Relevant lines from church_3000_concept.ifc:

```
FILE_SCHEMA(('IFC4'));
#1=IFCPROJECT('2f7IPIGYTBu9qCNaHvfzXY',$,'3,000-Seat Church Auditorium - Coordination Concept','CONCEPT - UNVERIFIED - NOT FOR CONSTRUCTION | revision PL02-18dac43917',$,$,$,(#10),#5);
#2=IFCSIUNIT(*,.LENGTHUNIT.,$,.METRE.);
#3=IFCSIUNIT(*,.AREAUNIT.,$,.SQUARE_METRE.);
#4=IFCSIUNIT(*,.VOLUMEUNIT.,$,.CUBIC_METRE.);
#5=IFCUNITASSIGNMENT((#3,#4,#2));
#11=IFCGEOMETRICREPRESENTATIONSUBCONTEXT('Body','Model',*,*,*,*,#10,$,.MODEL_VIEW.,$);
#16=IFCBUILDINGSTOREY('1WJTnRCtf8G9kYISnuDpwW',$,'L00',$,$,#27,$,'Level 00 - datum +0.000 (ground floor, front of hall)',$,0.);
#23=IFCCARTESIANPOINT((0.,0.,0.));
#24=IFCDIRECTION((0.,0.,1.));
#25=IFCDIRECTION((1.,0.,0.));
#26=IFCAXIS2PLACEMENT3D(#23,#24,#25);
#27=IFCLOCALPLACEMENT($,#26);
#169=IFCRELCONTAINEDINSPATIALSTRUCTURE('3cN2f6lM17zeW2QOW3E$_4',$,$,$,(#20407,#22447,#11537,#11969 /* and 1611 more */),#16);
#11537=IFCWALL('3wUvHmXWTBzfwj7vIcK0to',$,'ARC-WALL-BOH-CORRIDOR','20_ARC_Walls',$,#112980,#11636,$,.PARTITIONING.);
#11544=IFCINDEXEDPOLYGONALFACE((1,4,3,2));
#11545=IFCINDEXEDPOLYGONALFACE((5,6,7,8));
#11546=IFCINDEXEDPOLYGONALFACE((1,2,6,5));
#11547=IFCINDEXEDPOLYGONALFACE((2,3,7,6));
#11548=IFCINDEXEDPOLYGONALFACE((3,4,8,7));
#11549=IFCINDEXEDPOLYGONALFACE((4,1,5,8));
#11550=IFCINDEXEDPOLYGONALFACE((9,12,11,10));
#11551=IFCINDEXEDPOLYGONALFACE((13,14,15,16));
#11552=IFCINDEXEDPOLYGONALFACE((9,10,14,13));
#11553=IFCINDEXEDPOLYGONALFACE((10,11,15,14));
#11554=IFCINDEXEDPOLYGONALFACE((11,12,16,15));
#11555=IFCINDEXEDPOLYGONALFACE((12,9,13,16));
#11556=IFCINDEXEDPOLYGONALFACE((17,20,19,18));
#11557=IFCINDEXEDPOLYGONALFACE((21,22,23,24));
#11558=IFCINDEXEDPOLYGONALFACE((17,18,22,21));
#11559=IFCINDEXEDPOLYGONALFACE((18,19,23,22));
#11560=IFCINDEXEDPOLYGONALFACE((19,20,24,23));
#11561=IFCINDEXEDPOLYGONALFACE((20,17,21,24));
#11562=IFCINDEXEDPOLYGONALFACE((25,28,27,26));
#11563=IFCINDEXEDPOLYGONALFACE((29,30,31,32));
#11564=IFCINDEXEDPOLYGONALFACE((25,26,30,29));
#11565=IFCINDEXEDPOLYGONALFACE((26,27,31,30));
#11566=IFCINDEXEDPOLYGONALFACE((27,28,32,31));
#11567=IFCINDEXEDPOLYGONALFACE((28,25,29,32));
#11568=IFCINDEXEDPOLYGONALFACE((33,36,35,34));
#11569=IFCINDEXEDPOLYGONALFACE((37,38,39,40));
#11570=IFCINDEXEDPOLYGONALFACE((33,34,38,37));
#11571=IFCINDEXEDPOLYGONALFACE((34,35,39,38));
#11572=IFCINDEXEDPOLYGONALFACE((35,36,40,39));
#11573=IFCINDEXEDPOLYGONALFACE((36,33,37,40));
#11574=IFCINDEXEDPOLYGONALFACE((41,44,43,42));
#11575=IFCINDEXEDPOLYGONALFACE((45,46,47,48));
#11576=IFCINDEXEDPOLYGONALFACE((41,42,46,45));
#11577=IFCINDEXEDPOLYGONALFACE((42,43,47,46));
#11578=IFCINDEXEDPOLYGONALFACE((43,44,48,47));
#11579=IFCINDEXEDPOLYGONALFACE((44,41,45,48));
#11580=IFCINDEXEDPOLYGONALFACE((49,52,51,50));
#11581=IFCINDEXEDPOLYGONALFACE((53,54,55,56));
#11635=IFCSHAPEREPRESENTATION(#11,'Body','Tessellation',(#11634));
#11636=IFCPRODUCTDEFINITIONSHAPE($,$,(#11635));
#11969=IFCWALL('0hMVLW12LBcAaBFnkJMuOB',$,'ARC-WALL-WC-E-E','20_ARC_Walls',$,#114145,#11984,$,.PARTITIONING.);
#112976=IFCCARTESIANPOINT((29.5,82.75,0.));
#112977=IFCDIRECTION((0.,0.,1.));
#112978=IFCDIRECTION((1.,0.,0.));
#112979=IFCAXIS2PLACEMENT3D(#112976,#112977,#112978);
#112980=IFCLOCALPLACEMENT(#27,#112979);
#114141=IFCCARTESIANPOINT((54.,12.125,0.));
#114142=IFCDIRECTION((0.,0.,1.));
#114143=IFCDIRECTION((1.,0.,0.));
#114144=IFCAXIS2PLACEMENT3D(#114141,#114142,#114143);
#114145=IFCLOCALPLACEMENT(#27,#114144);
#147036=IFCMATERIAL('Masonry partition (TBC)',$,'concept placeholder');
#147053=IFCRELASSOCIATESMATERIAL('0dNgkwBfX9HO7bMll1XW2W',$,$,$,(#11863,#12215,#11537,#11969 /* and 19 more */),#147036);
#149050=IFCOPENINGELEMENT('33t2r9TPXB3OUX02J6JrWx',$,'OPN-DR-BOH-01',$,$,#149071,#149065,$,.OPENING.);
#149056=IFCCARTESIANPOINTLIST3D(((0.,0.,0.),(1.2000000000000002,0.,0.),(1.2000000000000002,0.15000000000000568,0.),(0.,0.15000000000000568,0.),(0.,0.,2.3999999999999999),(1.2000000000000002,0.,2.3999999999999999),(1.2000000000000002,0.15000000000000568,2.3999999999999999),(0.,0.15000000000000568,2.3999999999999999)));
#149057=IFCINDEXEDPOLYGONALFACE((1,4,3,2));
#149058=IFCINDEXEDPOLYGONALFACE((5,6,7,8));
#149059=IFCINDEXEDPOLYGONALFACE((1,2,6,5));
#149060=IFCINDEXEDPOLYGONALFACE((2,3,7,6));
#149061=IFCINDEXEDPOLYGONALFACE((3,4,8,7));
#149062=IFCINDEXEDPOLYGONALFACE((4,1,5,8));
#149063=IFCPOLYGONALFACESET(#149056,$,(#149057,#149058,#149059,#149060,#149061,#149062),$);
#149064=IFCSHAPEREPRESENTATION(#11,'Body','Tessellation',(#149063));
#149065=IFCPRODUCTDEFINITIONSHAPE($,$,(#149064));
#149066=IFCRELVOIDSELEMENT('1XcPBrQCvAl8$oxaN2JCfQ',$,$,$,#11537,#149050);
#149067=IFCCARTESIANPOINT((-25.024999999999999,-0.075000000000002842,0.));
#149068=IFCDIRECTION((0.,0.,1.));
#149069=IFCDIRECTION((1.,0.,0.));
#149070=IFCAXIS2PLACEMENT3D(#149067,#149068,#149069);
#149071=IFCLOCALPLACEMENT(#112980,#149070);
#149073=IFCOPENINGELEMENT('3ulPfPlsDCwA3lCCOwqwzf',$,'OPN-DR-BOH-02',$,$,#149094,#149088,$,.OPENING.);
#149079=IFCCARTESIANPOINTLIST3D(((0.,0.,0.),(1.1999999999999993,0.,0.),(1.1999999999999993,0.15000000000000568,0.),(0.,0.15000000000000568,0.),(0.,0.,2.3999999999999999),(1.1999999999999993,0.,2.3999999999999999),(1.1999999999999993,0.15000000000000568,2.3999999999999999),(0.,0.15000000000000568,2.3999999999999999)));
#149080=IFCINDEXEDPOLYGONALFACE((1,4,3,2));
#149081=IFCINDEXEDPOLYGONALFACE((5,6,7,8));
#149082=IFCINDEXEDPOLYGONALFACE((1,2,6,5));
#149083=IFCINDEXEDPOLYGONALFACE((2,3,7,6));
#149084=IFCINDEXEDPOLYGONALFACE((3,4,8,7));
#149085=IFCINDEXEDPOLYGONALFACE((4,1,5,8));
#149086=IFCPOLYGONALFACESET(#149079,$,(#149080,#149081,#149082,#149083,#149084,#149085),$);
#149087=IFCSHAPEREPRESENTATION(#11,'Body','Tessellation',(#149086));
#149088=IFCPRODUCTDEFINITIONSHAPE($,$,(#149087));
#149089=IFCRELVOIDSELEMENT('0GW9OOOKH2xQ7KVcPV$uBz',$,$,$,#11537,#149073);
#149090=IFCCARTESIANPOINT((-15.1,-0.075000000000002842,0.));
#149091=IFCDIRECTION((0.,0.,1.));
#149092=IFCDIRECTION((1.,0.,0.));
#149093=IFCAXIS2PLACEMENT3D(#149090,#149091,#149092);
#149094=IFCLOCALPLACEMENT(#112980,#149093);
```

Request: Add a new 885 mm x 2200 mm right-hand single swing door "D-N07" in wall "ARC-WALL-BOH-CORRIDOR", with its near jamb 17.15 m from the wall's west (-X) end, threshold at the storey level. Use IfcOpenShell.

```python
import numpy as np
import ifcopenshell
import ifcopenshell.api.feature
import ifcopenshell.api.geometry
import ifcopenshell.api.root
import ifcopenshell.api.spatial
import ifcopenshell.geom
import ifcopenshell.util.element
import ifcopenshell.util.placement
import ifcopenshell.util.representation
import ifcopenshell.util.shape
import ifcopenshell.util.unit

model = ifcopenshell.open("church_3000_concept.ifc")
unit_scale = ifcopenshell.util.unit.calculate_unit_scale(model)
settings = ifcopenshell.geom.settings()


def volume(element):
    """Net volume in cubic metres, openings subtracted."""
    shape = ifcopenshell.geom.create_shape(settings, element)
    return ifcopenshell.util.shape.get_volume(shape.geometry)


wall = model.by_guid("3wUvHmXWTBzfwj7vIcK0to")
storey = ifcopenshell.util.element.get_container(wall, ifc_class="IfcBuildingStorey")
context = ifcopenshell.util.representation.get_context(model, "Model", "Body", "MODEL_VIEW")
before = volume(wall)

width, height, from_end, sill = 0.885, 2.2, 17.15, 0.0  # metres

# The wall runs along its own X axis, and the end named is its -X end.
wall_shape = ifcopenshell.geom.create_shape(settings, wall)
x, y, z = ifcopenshell.util.shape.get_vertices(wall_shape.geometry).T
start = x.min() + from_end
face, thickness = float(y.min()), float(y.max() - y.min())
wall_matrix = ifcopenshell.util.placement.get_local_placement(wall.ObjectPlacement)
level = ifcopenshell.util.placement.get_local_placement(storey.ObjectPlacement)[2, 3]


def in_wall(x, y):
    """Placement at x, y metres in the wall's axes, at sill height."""
    matrix = wall_matrix.copy()
    matrix[:, 3] = wall_matrix @ np.array([x / unit_scale, y / unit_scale, 0.0, 1.0])
    matrix[2, 3] = level + sill / unit_scale
    return matrix


# Opening: a box that overshoots both wall faces by 50 mm.
opening = ifcopenshell.api.root.create_entity(model, ifc_class="IfcOpeningElement", predefined_type="OPENING")
box = ifcopenshell.api.geometry.add_wall_representation(
    model, context=context, length=width, height=height, thickness=thickness + 0.1
)
ifcopenshell.api.geometry.assign_representation(model, product=opening, representation=box)
ifcopenshell.api.geometry.edit_object_placement(model, product=opening, matrix=in_wall(start, face - 0.05), is_si=False)
ifcopenshell.api.feature.add_feature(model, feature=opening, element=wall)

door = ifcopenshell.api.root.create_entity(model, ifc_class="IfcDoor", name="D-N07", predefined_type="DOOR")
door.OverallWidth, door.OverallHeight = width / unit_scale, height / unit_scale
door.OperationType = "SINGLE_SWING_RIGHT"
body = ifcopenshell.api.geometry.add_door_representation(
    model,
    context=context,
    overall_width=door.OverallWidth,
    overall_height=door.OverallHeight,
    operation_type="SINGLE_SWING_RIGHT",
    lining_properties={"LiningDepth": thickness / unit_scale, "ThresholdDepth": thickness / unit_scale},
)
ifcopenshell.api.geometry.assign_representation(model, product=door, representation=body)
ifcopenshell.api.spatial.assign_container(model, products=[door], relating_structure=storey)
ifcopenshell.api.feature.add_filling(model, opening=opening, element=door)

# The lining spans the wall, so the door starts at the wall face.
ifcopenshell.api.geometry.edit_object_placement(model, product=door, matrix=in_wall(start, face), is_si=False)

after = volume(wall)

print(f"wall volume {before:.3f} -> {after:.3f} m3")

model.write("church_3000_concept_edited.ifc")
```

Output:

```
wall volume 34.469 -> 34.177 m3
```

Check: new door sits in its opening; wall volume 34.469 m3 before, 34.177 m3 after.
